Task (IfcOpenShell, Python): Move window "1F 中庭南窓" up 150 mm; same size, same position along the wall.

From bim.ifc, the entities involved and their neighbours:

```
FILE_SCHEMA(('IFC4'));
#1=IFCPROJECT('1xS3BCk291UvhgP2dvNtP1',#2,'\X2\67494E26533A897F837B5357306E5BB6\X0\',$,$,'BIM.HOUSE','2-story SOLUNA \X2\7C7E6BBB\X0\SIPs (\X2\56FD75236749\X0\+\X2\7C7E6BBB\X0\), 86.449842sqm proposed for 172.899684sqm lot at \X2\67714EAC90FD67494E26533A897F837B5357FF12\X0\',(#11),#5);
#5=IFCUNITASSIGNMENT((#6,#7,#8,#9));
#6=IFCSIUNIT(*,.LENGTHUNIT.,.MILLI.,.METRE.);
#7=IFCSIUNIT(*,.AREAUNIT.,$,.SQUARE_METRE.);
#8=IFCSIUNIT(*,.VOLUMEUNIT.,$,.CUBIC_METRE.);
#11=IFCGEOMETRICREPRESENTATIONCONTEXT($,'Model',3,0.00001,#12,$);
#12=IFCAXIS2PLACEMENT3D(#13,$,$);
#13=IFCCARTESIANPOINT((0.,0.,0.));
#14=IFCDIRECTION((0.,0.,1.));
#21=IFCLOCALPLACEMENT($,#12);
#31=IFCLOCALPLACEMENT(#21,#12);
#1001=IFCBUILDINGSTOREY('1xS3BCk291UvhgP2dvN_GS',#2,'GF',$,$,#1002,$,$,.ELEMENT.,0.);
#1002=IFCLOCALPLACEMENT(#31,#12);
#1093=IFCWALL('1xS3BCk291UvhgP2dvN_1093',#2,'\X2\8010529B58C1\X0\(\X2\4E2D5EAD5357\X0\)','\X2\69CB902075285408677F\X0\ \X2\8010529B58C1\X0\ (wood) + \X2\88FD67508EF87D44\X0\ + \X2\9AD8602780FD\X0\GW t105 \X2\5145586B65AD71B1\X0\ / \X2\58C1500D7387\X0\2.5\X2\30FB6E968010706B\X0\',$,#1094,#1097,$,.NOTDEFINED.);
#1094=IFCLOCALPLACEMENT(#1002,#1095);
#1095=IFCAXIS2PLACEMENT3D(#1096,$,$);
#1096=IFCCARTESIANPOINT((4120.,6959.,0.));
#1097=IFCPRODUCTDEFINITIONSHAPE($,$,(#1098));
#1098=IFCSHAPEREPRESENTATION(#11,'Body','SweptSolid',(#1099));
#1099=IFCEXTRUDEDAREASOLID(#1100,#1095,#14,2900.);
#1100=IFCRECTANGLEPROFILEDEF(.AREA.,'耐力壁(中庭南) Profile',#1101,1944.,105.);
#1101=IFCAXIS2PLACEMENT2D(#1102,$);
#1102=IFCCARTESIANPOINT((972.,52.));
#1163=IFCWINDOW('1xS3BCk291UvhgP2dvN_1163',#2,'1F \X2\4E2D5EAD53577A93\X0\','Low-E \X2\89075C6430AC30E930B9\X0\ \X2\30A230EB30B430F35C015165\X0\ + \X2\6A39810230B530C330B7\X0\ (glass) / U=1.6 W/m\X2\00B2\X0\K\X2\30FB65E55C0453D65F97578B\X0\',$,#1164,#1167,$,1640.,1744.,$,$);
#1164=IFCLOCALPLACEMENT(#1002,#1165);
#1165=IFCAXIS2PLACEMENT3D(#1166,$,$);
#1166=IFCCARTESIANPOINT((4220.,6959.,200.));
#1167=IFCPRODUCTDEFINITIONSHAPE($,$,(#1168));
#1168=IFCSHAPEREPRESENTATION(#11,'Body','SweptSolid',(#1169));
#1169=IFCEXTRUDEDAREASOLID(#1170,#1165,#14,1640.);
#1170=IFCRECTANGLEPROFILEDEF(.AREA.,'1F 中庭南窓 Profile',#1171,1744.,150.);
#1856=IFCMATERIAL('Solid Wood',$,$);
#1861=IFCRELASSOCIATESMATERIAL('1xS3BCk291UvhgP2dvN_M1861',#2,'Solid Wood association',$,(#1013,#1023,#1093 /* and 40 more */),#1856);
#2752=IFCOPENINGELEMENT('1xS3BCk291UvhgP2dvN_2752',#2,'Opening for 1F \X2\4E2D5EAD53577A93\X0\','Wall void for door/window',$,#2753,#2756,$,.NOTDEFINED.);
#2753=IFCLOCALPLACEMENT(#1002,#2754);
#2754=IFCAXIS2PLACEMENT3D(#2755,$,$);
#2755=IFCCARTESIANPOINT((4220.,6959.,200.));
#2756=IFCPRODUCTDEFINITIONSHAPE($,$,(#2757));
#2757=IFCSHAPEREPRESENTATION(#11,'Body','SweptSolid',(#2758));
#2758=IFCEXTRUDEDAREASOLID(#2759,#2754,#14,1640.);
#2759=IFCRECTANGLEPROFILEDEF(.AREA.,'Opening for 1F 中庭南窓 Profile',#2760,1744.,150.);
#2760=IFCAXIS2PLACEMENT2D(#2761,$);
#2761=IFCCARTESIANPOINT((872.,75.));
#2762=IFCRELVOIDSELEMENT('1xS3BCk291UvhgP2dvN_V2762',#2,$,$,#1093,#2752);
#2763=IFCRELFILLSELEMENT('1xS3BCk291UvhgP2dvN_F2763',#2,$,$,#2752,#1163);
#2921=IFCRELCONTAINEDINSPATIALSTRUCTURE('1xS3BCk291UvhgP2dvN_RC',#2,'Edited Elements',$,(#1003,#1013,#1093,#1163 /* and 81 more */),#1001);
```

```python
import numpy as np
import ifcopenshell
import ifcopenshell.api.geometry
import ifcopenshell.util.placement
import ifcopenshell.util.unit

model = ifcopenshell.open("bim.ifc")
unit_scale = ifcopenshell.util.unit.calculate_unit_scale(model)

window = model.by_guid("1xS3BCk291UvhgP2dvN_1163")
opening = window.FillsVoids[0].RelatingOpeningElement
dz = 150.0

shift = np.array([0.0, 0.0, dz])
# The window is not placed relative to its opening, so move both.
for product in (opening, window):
    matrix = ifcopenshell.util.placement.get_local_placement(product.ObjectPlacement)
    matrix[:3, 3] += shift
    ifcopenshell.api.geometry.edit_object_placement(model, product=product, matrix=matrix, is_si=False)

print(f"moved by {dz * unit_scale:+.3f} m")

model.write("bim-out.ifc")
```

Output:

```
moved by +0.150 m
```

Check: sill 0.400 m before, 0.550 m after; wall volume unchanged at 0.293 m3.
